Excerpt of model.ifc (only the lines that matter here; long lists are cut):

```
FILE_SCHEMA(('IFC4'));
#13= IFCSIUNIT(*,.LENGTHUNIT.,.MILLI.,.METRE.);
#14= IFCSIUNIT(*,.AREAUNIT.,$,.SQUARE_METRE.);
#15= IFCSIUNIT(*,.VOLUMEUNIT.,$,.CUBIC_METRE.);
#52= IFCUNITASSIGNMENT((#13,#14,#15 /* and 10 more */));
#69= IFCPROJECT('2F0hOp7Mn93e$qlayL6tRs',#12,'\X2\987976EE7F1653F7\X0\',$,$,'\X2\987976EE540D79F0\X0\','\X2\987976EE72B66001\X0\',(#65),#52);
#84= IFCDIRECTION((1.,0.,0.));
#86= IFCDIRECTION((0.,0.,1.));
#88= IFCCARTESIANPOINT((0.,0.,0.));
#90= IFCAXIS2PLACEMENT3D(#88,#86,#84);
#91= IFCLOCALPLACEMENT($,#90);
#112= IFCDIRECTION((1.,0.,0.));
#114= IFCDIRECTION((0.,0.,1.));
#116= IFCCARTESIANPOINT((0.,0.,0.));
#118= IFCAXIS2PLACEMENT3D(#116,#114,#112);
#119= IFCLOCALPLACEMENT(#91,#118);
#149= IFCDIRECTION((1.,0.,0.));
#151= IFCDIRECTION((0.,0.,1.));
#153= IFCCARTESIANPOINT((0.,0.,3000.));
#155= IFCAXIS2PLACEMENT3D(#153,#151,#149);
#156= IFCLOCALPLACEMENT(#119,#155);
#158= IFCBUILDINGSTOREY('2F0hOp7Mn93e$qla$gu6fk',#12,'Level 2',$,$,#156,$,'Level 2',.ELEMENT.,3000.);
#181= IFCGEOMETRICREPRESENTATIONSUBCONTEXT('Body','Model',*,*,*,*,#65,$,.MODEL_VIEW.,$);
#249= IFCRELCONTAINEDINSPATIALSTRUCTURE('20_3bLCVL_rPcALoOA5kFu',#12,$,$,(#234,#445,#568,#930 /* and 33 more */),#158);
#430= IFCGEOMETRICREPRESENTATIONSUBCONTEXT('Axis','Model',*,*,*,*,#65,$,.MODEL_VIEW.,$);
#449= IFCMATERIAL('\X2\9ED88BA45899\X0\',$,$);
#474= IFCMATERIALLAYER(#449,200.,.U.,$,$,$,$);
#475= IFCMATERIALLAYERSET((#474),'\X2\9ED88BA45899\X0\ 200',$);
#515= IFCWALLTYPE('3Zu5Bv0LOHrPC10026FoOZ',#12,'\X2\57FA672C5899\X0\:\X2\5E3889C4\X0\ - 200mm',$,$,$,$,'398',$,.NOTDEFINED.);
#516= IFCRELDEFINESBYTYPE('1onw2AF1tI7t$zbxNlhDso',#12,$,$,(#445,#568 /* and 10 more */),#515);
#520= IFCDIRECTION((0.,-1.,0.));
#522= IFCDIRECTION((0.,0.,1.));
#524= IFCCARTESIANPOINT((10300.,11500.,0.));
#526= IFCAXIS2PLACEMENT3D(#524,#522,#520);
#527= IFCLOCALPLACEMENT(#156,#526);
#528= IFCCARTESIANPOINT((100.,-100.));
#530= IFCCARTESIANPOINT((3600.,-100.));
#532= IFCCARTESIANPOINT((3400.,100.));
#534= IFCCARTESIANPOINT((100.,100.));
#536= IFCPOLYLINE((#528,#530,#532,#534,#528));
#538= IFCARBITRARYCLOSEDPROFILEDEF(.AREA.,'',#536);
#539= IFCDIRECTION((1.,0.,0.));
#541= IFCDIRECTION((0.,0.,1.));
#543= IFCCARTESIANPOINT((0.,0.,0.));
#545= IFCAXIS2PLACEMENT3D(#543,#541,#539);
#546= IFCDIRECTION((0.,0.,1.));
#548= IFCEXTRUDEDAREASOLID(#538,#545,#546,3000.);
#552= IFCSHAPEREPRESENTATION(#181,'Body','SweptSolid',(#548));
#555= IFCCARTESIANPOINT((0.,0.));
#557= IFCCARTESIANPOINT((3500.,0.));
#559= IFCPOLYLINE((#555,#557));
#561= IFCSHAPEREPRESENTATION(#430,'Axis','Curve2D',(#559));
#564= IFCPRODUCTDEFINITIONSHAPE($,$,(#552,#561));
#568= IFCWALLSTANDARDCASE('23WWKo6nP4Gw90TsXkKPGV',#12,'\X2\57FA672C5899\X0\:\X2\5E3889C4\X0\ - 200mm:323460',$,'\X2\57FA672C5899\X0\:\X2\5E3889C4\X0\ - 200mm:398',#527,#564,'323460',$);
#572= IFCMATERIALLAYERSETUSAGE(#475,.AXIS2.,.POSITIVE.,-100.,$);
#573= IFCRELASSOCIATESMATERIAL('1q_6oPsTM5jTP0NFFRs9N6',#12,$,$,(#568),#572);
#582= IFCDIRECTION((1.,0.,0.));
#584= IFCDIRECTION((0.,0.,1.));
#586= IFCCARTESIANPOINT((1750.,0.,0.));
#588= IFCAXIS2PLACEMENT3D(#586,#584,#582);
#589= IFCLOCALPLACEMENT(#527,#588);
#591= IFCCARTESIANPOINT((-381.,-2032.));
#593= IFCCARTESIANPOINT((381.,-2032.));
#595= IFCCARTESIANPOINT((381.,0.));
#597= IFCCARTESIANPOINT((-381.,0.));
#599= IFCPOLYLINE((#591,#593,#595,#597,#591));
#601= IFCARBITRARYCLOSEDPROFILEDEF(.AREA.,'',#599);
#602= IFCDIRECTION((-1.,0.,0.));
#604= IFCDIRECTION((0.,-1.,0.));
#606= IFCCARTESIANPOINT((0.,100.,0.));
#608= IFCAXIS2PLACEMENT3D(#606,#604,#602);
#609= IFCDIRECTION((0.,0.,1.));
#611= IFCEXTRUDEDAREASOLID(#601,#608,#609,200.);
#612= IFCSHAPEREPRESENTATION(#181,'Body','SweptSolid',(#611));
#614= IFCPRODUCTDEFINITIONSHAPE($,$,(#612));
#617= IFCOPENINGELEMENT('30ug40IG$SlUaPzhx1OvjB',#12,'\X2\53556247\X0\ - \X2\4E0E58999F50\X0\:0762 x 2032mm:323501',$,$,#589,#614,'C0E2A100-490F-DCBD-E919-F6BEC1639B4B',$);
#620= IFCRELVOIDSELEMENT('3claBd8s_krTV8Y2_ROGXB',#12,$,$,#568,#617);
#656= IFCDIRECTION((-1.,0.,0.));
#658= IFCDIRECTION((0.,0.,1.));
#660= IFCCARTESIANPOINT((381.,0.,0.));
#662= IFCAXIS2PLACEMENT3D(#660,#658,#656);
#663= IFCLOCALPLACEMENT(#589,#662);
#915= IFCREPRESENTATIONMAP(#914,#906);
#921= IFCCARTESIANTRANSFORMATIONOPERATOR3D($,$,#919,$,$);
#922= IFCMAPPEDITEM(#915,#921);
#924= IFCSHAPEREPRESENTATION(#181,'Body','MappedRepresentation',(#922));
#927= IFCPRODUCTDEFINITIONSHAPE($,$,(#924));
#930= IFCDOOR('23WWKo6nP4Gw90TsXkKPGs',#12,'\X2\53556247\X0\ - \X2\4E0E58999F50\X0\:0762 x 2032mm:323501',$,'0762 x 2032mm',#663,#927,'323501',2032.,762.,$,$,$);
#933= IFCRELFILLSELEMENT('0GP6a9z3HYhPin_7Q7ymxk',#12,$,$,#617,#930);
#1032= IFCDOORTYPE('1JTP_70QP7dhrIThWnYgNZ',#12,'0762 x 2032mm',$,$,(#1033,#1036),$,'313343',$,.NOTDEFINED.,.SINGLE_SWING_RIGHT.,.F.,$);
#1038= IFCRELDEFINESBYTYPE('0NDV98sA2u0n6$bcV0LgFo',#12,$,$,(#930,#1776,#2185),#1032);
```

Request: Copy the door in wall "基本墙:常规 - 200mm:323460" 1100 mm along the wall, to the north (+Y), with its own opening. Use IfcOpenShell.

```python
import ifcopenshell
import ifcopenshell.api.feature
import ifcopenshell.api.geometry
import ifcopenshell.api.root
import ifcopenshell.geom
import ifcopenshell.util.element
import ifcopenshell.util.placement
import ifcopenshell.util.shape
import ifcopenshell.util.unit

model = ifcopenshell.open("model.ifc")
unit_scale = ifcopenshell.util.unit.calculate_unit_scale(model)
settings = ifcopenshell.geom.settings()


def volume(element):
    """Net volume in cubic metres, openings subtracted."""
    shape = ifcopenshell.geom.create_shape(settings, element)
    return ifcopenshell.util.shape.get_volume(shape.geometry)


def reuse_history(source, copy):
    """copy_class also copies each property set's owner history, people and application; keep the originals."""
    for rel in copy.IsDefinedBy:
        if rel.is_a("IfcRelDefinesByProperties") and (history := rel.RelatingPropertyDefinition.OwnerHistory):
            rel.RelatingPropertyDefinition.OwnerHistory = source.OwnerHistory
            ifcopenshell.util.element.remove_deep2(model, history)


door = model.by_guid("23WWKo6nP4Gw90TsXkKPGs")
opening = door.FillsVoids[0].RelatingOpeningElement
wall = opening.VoidsElements[0].RelatingBuildingElement
before = volume(wall)
shift = ifcopenshell.util.placement.get_local_placement(wall.ObjectPlacement)[:3, 0] * -1.1 / unit_scale

# copy_class copies the void relationship, type, container and properties, but no geometry.
new_opening = ifcopenshell.api.root.copy_class(model, product=opening)
new_opening.Representation = ifcopenshell.util.element.copy_deep(
    model, opening.Representation, exclude=["IfcGeometricRepresentationContext", "IfcRepresentationMap"]
)
new_opening.Name = "单扇 - 与墙齐:0762 x 2032mm"
new_opening.Tag = None
new_door = ifcopenshell.api.root.copy_class(model, product=door)
new_door.Representation = ifcopenshell.util.element.copy_deep(
    model, door.Representation, exclude=["IfcGeometricRepresentationContext", "IfcRepresentationMap"]
)
new_door.Name = "单扇 - 与墙齐:0762 x 2032mm"
new_door.Tag = None
reuse_history(door, new_door)
ifcopenshell.api.feature.add_filling(model, opening=new_opening, element=new_door)

for old, new in ((opening, new_opening), (door, new_door)):
    matrix = ifcopenshell.util.placement.get_local_placement(old.ObjectPlacement)
    matrix[:3, 3] += shift
    ifcopenshell.api.geometry.edit_object_placement(model, product=new, matrix=matrix, is_si=False)

after = volume(wall)

print(f"wall volume {before:.3f} -> {after:.3f} m3")

model.write("model_updated.ifc")
```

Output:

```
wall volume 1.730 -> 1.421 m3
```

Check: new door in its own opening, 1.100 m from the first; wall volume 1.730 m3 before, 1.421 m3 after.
